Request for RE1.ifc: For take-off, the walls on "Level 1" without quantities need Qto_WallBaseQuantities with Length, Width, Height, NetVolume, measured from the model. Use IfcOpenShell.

First a look at what the model holds.

```python
import ifcopenshell
import ifcopenshell.util.element
import ifcopenshell.util.unit

model = ifcopenshell.open("RE1.ifc")
print(model.schema)
for unit_type in ("LENGTHUNIT", "AREAUNIT", "VOLUMEUNIT"):
    print(unit_type, ifcopenshell.util.unit.calculate_unit_scale(model, unit_type))
storey = next(s for s in model.by_type("IfcBuildingStorey") if s.Name == "Level 1")
walls = [e for e in ifcopenshell.util.element.get_decomposition(storey) if e.is_a("IfcWall")]
for e in sorted(walls, key=lambda e: e.id()):
    print(e.id(), e.is_a(), e.Name, list(ifcopenshell.util.element.get_psets(e, qtos_only=True)), sep=" | ")
```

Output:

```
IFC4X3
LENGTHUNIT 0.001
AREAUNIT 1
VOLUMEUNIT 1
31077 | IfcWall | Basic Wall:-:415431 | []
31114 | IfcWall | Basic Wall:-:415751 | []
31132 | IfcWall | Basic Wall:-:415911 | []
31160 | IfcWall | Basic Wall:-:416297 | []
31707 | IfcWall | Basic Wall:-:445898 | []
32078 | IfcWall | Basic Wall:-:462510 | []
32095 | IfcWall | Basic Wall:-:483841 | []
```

```python
import ifcopenshell
import ifcopenshell.api.pset
import ifcopenshell.geom
import ifcopenshell.util.element
import ifcopenshell.util.shape
import ifcopenshell.util.unit

model = ifcopenshell.open("RE1.ifc")
unit_scale = ifcopenshell.util.unit.calculate_unit_scale(model)
volume_scale = ifcopenshell.util.unit.calculate_unit_scale(model, "VOLUMEUNIT")
settings = ifcopenshell.geom.settings()

storey = next(s for s in model.by_type("IfcBuildingStorey") if s.Name == "Level 1")
walls = [e for e in ifcopenshell.util.element.get_decomposition(storey) if e.is_a("IfcWall")]

for e in sorted(walls, key=lambda e: e.id()):
    if ifcopenshell.util.element.get_psets(e, qtos_only=True, should_inherit=False):
        continue
    # Geometry comes back in metres, in the element's own axes.
    shape = ifcopenshell.geom.create_shape(settings, e)
    values = {
        "Length": ifcopenshell.util.shape.get_x(shape.geometry) / unit_scale,
        "Width": ifcopenshell.util.shape.get_y(shape.geometry) / unit_scale,
        "Height": ifcopenshell.util.shape.get_z(shape.geometry) / unit_scale,
        "NetVolume": ifcopenshell.util.shape.get_volume(shape.geometry) / volume_scale,
    }
    qto = ifcopenshell.api.pset.add_qto(model, product=e, name="Qto_WallBaseQuantities")
    ifcopenshell.api.pset.edit_qto(model, qto=qto, properties=values)
    print(e.id(), {k: round(v, 3) for k, v in values.items()})

model.write("RE1_v2.ifc")
```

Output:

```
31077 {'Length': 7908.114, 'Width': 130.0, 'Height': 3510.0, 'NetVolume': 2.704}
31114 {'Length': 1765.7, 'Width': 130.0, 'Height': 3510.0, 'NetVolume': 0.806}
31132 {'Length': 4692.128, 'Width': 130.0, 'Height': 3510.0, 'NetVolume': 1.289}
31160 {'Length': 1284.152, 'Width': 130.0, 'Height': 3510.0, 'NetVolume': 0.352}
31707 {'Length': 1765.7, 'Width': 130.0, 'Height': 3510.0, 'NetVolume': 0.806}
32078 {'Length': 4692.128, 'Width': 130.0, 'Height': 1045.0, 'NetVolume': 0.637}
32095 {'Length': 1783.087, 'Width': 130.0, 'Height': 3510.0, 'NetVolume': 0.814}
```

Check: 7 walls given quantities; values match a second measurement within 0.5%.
